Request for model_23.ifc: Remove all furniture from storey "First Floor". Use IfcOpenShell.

First a look at what the model holds.

```python
import ifcopenshell
import ifcopenshell.util.element

model = ifcopenshell.open("model_23.ifc")
print(model.schema)
storey = next(s for s in model.by_type("IfcBuildingStorey") if s.Name == "First Floor")
furniture = [e for e in ifcopenshell.util.element.get_decomposition(storey) if e.is_a("IfcFurnishingElement")]
seen = {}
for e in furniture:
    element_type = ifcopenshell.util.element.get_type(e)
    name = element_type.Name if element_type not in (None, e) else None
    seen[name] = seen.get(name, 0) + 1
for name, count in sorted(seen.items(), key=str):
    print(count, "x", name)
```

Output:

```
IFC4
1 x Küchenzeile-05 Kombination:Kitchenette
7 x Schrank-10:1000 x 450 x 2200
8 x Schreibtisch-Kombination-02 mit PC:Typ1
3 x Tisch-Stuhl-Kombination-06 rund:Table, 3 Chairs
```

```python
import ifcopenshell
import ifcopenshell.api.root
import ifcopenshell.util.element

model = ifcopenshell.open("model_23.ifc")

storey = next(s for s in model.by_type("IfcBuildingStorey") if s.Name == "First Floor")
furniture = [e for e in ifcopenshell.util.element.get_decomposition(storey) if e.is_a("IfcFurnishingElement")]

for e in furniture:
    ifcopenshell.api.root.remove_product(model, product=e)
print(len(furniture), "removed")

model.write("model_23_updated.ifc")
```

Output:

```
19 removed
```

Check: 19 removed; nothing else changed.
